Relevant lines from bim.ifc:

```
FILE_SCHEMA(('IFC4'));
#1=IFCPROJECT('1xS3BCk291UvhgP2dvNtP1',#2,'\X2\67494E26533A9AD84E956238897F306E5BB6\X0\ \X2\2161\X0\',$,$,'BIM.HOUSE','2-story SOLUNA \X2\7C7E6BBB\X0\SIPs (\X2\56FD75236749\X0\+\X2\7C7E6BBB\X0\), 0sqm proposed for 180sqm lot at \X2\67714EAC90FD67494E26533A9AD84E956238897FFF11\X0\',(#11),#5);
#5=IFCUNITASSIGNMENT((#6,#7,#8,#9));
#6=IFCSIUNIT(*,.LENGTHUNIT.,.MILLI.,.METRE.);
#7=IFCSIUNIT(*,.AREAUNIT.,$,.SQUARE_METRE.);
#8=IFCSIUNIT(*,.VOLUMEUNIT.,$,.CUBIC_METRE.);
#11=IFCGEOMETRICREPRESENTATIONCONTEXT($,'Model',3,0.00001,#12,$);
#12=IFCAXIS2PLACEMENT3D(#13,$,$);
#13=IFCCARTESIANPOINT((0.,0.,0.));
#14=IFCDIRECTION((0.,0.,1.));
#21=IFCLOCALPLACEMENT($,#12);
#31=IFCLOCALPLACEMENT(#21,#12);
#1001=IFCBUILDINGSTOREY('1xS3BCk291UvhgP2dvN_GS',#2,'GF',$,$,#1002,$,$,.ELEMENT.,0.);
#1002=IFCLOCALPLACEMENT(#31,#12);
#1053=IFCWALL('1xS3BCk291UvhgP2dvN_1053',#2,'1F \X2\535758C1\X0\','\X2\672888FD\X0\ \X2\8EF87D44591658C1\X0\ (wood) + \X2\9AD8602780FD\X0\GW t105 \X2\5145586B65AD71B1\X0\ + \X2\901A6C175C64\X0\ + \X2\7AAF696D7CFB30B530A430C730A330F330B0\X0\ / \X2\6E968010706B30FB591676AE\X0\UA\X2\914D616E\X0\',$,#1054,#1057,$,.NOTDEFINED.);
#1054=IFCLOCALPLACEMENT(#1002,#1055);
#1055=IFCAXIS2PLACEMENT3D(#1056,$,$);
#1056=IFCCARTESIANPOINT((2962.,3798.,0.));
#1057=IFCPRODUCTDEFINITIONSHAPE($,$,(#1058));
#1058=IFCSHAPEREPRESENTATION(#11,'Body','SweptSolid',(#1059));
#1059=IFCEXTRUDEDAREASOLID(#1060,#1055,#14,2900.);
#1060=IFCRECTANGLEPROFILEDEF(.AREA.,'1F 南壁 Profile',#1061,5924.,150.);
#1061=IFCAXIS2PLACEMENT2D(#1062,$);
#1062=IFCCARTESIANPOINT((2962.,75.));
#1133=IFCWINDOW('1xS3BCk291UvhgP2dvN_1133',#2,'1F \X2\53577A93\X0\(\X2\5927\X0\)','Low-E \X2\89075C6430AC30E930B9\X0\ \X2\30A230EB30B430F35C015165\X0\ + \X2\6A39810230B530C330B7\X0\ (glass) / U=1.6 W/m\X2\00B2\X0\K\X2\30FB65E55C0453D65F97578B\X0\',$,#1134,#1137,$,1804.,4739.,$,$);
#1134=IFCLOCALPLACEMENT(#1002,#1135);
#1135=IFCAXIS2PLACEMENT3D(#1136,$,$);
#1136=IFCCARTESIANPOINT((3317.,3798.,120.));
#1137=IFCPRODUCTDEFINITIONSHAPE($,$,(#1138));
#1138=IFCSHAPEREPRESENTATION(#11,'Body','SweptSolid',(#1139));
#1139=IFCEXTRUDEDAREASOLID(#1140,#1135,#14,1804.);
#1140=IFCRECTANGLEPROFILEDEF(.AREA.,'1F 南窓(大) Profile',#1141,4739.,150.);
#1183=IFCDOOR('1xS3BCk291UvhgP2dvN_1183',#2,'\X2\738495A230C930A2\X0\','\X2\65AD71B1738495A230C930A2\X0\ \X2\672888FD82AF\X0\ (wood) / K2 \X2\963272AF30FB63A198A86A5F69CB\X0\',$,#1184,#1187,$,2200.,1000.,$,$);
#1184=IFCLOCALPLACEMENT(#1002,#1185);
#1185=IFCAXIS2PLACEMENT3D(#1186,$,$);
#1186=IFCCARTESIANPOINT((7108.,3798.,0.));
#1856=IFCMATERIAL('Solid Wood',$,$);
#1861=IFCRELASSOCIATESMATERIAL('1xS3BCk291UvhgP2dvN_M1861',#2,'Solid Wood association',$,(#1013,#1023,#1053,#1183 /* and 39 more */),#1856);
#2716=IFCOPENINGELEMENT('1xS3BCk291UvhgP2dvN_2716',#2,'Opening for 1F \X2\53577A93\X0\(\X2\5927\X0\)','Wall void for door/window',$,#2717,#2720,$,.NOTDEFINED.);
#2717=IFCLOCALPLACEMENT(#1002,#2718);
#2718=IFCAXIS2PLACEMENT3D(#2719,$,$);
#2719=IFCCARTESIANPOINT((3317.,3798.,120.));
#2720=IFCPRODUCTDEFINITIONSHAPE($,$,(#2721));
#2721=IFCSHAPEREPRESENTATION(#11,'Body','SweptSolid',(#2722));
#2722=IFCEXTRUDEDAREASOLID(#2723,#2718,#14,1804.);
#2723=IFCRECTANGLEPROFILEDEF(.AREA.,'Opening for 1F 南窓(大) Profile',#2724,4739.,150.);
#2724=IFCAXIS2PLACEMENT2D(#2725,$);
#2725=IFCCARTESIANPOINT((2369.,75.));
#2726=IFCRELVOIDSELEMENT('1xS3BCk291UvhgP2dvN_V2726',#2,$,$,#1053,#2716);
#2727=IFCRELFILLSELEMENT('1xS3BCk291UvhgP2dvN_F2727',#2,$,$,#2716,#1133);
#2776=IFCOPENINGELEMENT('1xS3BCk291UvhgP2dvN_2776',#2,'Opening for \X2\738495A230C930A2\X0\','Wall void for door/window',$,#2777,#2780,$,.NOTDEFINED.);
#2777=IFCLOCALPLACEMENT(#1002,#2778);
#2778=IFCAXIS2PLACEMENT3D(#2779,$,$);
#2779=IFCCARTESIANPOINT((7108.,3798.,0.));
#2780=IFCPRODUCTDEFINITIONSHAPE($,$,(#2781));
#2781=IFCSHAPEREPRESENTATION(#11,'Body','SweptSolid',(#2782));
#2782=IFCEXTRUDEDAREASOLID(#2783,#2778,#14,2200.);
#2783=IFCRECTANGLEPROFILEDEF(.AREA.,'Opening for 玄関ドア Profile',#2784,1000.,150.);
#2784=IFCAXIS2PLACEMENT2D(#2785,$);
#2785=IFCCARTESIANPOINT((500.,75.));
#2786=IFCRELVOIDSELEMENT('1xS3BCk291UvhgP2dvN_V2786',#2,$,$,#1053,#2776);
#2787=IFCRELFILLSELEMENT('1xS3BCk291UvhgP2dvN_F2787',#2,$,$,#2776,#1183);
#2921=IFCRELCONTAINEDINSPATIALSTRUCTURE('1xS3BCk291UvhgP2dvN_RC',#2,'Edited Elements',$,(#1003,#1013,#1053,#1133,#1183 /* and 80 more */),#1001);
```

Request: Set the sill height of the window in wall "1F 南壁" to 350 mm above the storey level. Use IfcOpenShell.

```python
import numpy as np
import ifcopenshell
import ifcopenshell.api.geometry
import ifcopenshell.geom
import ifcopenshell.util.element
import ifcopenshell.util.placement
import ifcopenshell.util.shape
import ifcopenshell.util.unit

model = ifcopenshell.open("bim.ifc")
unit_scale = ifcopenshell.util.unit.calculate_unit_scale(model)

window = model.by_guid("1xS3BCk291UvhgP2dvN_1133")
opening = window.FillsVoids[0].RelatingOpeningElement
storey = ifcopenshell.util.element.get_container(window, ifc_class="IfcBuildingStorey")
level = ifcopenshell.util.placement.get_local_placement(storey.ObjectPlacement)[2, 3]

# The opening's origin need not be at the sill, so measure its lowest point.
shape = ifcopenshell.geom.create_shape(ifcopenshell.geom.settings(), opening)
bottom = ifcopenshell.util.shape.get_shape_bottom_elevation(shape, shape.geometry) / unit_scale
dz = level + 350.0 - bottom

shift = np.array([0.0, 0.0, dz])
# The window is not placed relative to its opening, so move both.
for product in (opening, window):
    matrix = ifcopenshell.util.placement.get_local_placement(product.ObjectPlacement)
    matrix[:3, 3] += shift
    ifcopenshell.api.geometry.edit_object_placement(model, product=product, matrix=matrix, is_si=False)

print(f"moved by {dz * unit_scale:+.3f} m")

model.write("bim_rev.ifc")
```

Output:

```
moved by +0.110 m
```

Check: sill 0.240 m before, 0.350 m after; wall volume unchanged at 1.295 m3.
